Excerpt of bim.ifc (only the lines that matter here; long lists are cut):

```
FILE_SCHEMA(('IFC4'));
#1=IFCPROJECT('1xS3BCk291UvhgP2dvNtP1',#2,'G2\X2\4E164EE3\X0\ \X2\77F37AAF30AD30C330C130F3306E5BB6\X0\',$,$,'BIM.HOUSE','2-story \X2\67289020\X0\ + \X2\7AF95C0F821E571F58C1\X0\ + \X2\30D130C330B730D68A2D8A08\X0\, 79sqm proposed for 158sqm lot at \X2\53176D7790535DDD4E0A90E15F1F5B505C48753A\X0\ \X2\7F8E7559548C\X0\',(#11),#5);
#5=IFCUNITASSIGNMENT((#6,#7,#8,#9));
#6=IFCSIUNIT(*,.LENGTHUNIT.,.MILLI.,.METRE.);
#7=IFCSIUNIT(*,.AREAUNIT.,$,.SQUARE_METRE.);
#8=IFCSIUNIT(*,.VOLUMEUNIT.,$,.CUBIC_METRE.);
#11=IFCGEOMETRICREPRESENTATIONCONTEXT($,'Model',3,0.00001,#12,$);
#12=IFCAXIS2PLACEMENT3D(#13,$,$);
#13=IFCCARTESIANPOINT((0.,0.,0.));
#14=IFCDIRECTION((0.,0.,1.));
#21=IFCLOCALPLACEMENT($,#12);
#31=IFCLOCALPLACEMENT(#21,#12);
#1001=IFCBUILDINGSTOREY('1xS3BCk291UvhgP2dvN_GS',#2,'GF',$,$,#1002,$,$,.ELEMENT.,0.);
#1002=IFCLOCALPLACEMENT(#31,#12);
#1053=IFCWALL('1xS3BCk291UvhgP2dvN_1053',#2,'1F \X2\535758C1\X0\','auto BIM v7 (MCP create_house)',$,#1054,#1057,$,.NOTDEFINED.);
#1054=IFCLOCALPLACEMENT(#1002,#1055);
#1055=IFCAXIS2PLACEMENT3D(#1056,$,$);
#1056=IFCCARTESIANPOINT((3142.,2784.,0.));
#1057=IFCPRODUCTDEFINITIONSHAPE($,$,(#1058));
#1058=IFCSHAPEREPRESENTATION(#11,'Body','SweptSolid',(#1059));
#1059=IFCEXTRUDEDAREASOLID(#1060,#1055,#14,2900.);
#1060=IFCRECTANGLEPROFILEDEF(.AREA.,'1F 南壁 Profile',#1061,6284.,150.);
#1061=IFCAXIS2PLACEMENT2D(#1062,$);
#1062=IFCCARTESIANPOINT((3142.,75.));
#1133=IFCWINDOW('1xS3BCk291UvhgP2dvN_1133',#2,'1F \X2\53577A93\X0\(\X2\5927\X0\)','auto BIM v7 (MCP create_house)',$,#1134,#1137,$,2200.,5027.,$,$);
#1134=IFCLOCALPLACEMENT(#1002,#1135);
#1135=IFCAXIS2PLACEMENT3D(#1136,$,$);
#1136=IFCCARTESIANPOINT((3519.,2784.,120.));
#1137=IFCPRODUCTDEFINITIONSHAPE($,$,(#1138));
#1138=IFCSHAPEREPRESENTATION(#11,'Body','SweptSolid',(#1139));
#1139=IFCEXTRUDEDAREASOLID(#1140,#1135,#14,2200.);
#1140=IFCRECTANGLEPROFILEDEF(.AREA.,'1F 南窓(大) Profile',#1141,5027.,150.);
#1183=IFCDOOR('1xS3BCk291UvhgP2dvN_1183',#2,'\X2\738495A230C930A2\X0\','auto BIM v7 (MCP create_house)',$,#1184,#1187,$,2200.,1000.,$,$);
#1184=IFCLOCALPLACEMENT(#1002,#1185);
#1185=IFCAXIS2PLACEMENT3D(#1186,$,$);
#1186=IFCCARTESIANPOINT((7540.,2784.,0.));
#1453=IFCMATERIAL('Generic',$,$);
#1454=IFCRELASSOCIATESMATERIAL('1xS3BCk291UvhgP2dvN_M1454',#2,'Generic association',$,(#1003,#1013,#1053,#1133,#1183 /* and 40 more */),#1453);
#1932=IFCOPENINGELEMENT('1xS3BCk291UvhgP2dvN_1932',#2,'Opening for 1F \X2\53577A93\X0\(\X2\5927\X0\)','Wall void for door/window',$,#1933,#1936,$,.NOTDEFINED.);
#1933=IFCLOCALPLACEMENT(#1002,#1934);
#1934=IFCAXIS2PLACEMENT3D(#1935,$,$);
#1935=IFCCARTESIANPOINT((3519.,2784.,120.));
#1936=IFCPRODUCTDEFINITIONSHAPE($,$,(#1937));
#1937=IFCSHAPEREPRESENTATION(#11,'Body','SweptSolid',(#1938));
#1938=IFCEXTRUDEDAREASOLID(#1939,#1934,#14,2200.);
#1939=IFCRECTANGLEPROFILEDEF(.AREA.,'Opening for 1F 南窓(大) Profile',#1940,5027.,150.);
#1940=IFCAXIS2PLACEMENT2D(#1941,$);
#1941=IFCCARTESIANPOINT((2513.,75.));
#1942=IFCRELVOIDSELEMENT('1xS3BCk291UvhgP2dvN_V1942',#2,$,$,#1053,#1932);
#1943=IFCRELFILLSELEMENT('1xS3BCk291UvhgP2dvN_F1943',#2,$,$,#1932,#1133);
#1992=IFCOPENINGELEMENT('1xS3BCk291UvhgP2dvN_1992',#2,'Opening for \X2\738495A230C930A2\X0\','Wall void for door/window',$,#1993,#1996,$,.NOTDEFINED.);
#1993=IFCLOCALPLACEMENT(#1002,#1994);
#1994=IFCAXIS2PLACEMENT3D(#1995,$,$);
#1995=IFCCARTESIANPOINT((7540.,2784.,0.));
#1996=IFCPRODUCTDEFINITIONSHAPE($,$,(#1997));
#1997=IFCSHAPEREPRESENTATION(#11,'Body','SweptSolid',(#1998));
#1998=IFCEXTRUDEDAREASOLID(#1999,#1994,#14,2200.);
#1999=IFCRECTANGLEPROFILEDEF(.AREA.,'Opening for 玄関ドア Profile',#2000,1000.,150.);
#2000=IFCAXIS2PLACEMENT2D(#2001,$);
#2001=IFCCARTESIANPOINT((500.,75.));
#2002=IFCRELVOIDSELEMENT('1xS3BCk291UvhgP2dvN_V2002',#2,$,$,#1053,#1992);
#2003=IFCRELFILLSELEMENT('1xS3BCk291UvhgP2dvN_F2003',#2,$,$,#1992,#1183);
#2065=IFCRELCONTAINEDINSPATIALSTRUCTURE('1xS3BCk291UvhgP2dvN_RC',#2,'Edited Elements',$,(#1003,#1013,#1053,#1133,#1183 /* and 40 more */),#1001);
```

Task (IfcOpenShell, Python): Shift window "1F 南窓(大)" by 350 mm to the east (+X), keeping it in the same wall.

```python
import ifcopenshell
import ifcopenshell.api.geometry
import ifcopenshell.util.placement
import ifcopenshell.util.unit

model = ifcopenshell.open("bim.ifc")
unit_scale = ifcopenshell.util.unit.calculate_unit_scale(model)

window = model.by_id(1133)
opening = window.FillsVoids[0].RelatingOpeningElement
wall = opening.VoidsElements[0].RelatingBuildingElement

wall_matrix = ifcopenshell.util.placement.get_local_placement(wall.ObjectPlacement)
shift = wall_matrix[:3, 0] * 0.35 / unit_scale
before = ifcopenshell.util.placement.get_local_placement(window.ObjectPlacement)[:3, 3].copy()

# The window is not placed relative to its opening, so move both.
for product in (opening, window):
    matrix = ifcopenshell.util.placement.get_local_placement(product.ObjectPlacement)
    matrix[:3, 3] += shift
    ifcopenshell.api.geometry.edit_object_placement(model, product=product, matrix=matrix, is_si=False)

after = ifcopenshell.util.placement.get_local_placement(window.ObjectPlacement)[:3, 3]
print("window moved by", (after - before).round(3) + 0.0)

model.write("bim_v2.ifc")
```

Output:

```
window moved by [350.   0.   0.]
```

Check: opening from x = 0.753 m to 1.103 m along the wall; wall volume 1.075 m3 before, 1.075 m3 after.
